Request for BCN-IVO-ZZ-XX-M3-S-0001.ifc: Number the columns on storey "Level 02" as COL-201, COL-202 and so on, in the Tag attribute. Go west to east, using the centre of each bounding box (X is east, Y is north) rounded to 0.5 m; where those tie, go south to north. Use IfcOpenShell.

First a look at what the model holds.

```python
import ifcopenshell
import ifcopenshell.util.element
import ifcopenshell.util.placement

model = ifcopenshell.open("BCN-IVO-ZZ-XX-M3-S-0001.ifc")
print(model.schema)
storey = next(s for s in model.by_type("IfcBuildingStorey") if s.Name == "Level 02")
columns = [e for e in ifcopenshell.util.element.get_decomposition(storey) if e.is_a("IfcColumn")]
for e in sorted(columns, key=lambda e: e.id()):
    origin = ifcopenshell.util.placement.get_local_placement(e.ObjectPlacement)[:3, 3]
    print(e.id(), e.Tag, e.Name, origin.round(2) + 0.0, sep=" | ")
```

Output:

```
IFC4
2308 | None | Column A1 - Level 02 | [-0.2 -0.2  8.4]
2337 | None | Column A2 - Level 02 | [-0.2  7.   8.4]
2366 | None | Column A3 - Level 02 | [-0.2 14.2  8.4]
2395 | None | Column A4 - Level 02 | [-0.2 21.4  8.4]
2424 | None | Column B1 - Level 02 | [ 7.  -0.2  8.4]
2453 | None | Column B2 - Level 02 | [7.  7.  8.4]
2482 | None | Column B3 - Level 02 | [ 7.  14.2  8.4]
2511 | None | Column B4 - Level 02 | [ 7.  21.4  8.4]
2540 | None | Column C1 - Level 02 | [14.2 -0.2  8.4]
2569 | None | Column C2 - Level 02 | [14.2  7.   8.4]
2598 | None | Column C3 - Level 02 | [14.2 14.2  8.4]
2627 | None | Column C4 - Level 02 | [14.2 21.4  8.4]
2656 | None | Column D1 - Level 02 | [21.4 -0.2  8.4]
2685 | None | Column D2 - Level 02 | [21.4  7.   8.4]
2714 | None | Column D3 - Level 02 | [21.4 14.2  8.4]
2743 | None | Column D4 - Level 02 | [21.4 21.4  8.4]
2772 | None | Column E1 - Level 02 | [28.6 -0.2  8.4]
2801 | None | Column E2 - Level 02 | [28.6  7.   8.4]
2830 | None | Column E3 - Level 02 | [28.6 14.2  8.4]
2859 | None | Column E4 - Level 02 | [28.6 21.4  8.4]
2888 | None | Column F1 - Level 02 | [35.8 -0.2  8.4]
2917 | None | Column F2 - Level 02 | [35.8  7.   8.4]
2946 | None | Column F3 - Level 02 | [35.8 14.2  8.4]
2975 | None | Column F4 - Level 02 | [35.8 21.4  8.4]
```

```python
import ifcopenshell
import ifcopenshell.geom
import ifcopenshell.util.element
import ifcopenshell.util.shape

model = ifcopenshell.open("BCN-IVO-ZZ-XX-M3-S-0001.ifc")
settings = ifcopenshell.geom.settings()
settings.set("use-world-coords", True)


def centre(element):
    shape = ifcopenshell.geom.create_shape(settings, element)
    return ifcopenshell.util.shape.get_bbox_centroid(shape.geometry)


storey = next(s for s in model.by_type("IfcBuildingStorey") if s.Name == "Level 02")
columns = [e for e in ifcopenshell.util.element.get_decomposition(storey) if e.is_a("IfcColumn")]

# Insertion points can sit at a corner or the storey origin, so sort by the geometry (in metres).
centres = {e: centre(e) for e in columns}
columns.sort(key=lambda e: (round(centres[e][0] / 0.5), centres[e][1]))

for i, e in enumerate(columns, start=1):
    number = f"COL-2{i:02d}"
    e.Tag = number
    print(e.id(), number)

model.write("BCN-IVO-ZZ-XX-M3-S-0001_edited.ifc")
```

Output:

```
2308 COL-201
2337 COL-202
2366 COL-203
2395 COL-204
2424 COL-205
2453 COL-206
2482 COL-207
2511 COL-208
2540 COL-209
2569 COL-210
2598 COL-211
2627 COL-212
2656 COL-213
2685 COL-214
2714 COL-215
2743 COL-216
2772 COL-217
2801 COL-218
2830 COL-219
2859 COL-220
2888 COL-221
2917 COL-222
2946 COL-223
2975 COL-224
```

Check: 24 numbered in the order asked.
